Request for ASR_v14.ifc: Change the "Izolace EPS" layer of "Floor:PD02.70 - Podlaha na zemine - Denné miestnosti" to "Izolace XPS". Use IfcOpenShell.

First a look at what the model holds.

```python
import ifcopenshell
import ifcopenshell.util.element

model = ifcopenshell.open("ASR_v14.ifc")
print(model.schema)
for layer_set in model.by_type("IfcMaterialLayerSet"):
    if layer_set.LayerSetName == "Floor:PD02.70 - Podlaha na zemine - Denné miestnosti":
        for layer in layer_set.MaterialLayers:
            print(layer.id(), layer.Material and layer.Material.Name, layer.LayerThickness, sep=" | ")
        print(len(ifcopenshell.util.element.get_elements_by_material(model, layer_set)), "elements and types use it")
print(sorted(m.Name for m in model.by_type("IfcMaterial") if m.Name)[:60])
```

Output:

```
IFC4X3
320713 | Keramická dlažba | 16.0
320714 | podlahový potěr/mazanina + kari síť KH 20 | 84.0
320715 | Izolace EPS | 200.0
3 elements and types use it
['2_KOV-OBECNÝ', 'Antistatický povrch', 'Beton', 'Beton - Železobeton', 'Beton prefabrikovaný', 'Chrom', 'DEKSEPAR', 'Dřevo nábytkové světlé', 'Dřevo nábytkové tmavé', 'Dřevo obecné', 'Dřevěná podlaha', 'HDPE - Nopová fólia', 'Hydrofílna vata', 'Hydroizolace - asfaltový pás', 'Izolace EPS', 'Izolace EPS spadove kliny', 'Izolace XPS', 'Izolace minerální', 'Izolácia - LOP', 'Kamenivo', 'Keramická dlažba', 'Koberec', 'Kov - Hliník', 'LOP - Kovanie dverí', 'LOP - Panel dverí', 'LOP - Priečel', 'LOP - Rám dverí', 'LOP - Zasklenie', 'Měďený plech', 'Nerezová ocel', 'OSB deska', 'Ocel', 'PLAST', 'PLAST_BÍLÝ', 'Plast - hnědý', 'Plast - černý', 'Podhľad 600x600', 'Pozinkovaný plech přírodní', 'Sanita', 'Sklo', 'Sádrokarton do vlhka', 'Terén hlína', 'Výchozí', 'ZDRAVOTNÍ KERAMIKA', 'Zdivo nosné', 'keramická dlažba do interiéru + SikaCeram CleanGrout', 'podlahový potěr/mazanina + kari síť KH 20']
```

```python
import ifcopenshell
import ifcopenshell.api.material

model = ifcopenshell.open("ASR_v14.ifc")

layer_set = next(s for s in model.by_type("IfcMaterialLayerSet") if s.LayerSetName == "Floor:PD02.70 - Podlaha na zemine - Denné miestnosti")
layer = next(l for l in layer_set.MaterialLayers if l.Material and l.Material.Name == "Izolace EPS")
material = next(m for m in model.by_type("IfcMaterial") if m.Name == "Izolace XPS")

# Point this one layer at the other material; renaming the old one would change it everywhere.
ifcopenshell.api.material.edit_layer(model, layer=layer, attributes={"Name": material.Name}, material=material)

print([l.Material.Name if l.Material else None for l in layer_set.MaterialLayers])

model.write("ASR_v14-out.ifc")
```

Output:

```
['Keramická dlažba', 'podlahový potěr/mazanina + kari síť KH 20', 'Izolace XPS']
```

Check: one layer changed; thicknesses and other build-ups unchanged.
